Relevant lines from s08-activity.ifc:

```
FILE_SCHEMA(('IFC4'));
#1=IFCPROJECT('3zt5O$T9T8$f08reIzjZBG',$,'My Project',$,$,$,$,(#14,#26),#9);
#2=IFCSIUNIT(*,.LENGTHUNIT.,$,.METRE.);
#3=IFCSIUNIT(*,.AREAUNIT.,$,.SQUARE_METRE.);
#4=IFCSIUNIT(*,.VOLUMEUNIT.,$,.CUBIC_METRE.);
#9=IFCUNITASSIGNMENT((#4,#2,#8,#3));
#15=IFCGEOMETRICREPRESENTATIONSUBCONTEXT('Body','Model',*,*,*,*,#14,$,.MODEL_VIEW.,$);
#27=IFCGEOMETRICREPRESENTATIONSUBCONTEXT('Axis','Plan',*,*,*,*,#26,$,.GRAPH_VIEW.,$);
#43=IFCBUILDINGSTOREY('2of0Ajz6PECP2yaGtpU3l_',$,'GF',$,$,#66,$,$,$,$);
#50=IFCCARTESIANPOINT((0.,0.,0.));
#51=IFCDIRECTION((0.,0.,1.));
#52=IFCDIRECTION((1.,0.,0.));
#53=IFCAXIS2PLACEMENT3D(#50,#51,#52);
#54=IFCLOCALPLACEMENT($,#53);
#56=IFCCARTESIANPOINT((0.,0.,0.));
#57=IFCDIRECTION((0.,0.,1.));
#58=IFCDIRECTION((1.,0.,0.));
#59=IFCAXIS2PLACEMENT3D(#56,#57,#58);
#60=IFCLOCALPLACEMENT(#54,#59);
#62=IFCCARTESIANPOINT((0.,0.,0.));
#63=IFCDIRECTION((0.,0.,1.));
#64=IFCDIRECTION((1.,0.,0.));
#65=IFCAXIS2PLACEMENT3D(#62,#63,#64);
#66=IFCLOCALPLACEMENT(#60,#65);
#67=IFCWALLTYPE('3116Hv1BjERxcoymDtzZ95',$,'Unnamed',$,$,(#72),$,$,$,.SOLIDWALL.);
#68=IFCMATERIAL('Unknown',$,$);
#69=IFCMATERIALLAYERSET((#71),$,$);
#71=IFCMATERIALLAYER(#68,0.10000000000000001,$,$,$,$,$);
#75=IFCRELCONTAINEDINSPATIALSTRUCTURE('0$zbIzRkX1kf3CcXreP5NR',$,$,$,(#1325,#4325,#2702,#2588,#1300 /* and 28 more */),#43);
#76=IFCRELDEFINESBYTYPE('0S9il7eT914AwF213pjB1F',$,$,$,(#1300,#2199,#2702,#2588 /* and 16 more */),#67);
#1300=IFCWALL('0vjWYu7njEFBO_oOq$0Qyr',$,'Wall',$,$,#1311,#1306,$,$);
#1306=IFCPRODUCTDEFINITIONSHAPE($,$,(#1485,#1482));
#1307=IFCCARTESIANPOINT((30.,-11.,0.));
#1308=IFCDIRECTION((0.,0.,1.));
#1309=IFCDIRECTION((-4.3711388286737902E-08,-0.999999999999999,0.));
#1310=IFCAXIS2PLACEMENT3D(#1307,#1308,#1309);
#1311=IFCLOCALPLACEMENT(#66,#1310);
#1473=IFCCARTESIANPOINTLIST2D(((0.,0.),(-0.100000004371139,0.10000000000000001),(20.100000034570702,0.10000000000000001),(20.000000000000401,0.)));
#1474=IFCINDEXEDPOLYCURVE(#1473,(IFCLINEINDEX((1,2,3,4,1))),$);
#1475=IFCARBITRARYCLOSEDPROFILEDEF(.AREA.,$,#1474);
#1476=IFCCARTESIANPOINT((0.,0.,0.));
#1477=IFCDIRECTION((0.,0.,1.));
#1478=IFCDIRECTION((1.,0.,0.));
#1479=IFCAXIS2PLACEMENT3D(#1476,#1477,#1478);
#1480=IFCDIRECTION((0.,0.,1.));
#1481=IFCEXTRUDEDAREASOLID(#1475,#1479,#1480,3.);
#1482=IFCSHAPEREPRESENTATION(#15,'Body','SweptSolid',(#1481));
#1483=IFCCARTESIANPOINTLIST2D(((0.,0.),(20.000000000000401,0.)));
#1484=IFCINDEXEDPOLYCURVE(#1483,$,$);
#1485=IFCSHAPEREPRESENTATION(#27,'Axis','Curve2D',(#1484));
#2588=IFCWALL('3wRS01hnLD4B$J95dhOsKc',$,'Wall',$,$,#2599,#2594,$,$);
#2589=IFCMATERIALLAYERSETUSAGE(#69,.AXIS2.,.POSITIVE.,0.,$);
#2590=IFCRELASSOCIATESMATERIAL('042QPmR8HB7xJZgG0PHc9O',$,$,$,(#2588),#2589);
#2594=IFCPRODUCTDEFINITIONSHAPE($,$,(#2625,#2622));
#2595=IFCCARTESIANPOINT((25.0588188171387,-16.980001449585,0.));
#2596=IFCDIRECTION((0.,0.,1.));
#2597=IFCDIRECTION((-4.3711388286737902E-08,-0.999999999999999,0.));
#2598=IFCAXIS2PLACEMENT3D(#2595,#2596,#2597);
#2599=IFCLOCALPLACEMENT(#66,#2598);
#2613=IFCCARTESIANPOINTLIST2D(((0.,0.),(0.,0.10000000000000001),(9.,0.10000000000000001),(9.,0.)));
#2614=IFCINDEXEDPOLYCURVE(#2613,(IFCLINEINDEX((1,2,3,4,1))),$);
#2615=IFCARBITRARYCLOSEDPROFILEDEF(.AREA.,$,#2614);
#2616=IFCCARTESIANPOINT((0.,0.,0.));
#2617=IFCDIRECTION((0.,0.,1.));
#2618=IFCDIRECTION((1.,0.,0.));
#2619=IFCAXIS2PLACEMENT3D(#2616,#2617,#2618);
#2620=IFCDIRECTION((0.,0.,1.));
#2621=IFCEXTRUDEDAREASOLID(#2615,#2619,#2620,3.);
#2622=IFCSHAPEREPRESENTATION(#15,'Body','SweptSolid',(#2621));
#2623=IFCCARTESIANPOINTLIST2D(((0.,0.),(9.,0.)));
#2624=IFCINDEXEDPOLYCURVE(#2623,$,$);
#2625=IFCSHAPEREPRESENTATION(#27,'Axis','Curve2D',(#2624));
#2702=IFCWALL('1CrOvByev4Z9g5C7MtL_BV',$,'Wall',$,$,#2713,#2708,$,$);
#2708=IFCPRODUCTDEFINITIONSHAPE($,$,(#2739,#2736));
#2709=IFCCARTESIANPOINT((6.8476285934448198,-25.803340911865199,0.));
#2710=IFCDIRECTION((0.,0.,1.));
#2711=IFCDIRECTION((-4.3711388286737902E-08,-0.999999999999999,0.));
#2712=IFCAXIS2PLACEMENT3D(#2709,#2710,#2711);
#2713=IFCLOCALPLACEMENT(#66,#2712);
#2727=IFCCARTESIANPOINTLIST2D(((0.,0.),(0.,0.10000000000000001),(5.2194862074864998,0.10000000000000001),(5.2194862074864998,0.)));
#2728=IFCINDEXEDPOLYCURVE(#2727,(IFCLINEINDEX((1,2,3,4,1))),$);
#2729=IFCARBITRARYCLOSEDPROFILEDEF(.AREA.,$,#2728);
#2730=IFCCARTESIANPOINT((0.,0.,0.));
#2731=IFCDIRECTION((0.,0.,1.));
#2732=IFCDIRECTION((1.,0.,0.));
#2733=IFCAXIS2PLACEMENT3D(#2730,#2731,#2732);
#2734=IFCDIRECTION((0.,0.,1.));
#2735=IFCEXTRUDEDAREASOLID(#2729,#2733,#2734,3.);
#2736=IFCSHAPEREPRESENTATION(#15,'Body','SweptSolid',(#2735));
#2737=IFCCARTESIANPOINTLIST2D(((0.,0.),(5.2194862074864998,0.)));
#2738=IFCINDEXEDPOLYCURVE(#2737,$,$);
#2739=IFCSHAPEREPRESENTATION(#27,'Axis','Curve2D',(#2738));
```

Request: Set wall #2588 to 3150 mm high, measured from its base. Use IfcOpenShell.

```python
import ifcopenshell
import ifcopenshell.geom
import ifcopenshell.util.representation
import ifcopenshell.util.shape
import ifcopenshell.util.unit

model = ifcopenshell.open("s08-activity.ifc")
unit_scale = ifcopenshell.util.unit.calculate_unit_scale(model)
settings = ifcopenshell.geom.settings()


def volume(element):
    """Net volume in cubic metres, openings subtracted."""
    shape = ifcopenshell.geom.create_shape(settings, element)
    return ifcopenshell.util.shape.get_volume(shape.geometry)


wall = model.by_guid("3wRS01hnLD4B$J95dhOsKc")
before = volume(wall)

body = ifcopenshell.util.representation.get_representation(wall, "Model", "Body")
solid = body.Items[0]
old_height = solid.Depth
solid.Depth = 3.15 / unit_scale
after = volume(wall)

print(f"height {old_height:g} -> {solid.Depth:g}, volume {before:.3f} -> {after:.3f} m3")

model.write("s08-activity_updated.ifc")
```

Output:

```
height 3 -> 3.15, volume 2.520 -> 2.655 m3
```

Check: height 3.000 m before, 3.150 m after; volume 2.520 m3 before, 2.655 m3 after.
